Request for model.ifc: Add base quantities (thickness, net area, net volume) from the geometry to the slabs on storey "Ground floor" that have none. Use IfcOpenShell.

First a look at what the model holds.

```python
import ifcopenshell
import ifcopenshell.util.element
import ifcopenshell.util.unit

model = ifcopenshell.open("model.ifc")
print(model.schema)
for unit_type in ("LENGTHUNIT", "AREAUNIT", "VOLUMEUNIT"):
    print(unit_type, ifcopenshell.util.unit.calculate_unit_scale(model, unit_type))
storey = next(s for s in model.by_type("IfcBuildingStorey") if s.Name == "Ground floor")
slabs = [e for e in ifcopenshell.util.element.get_decomposition(storey) if e.is_a("IfcSlab")]
for e in sorted(slabs, key=lambda e: e.id()):
    print(e.id(), e.is_a(), e.Name, list(ifcopenshell.util.element.get_psets(e, qtos_only=True)), sep=" | ")
```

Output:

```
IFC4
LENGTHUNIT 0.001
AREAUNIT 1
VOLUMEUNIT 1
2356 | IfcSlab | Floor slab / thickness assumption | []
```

```python
import ifcopenshell
import ifcopenshell.api.pset
import ifcopenshell.geom
import ifcopenshell.util.element
import ifcopenshell.util.shape
import ifcopenshell.util.unit

model = ifcopenshell.open("model.ifc")
unit_scale = ifcopenshell.util.unit.calculate_unit_scale(model)
area_scale = ifcopenshell.util.unit.calculate_unit_scale(model, "AREAUNIT")
volume_scale = ifcopenshell.util.unit.calculate_unit_scale(model, "VOLUMEUNIT")
settings = ifcopenshell.geom.settings()

storey = next(s for s in model.by_type("IfcBuildingStorey") if s.Name == "Ground floor")
slabs = [e for e in ifcopenshell.util.element.get_decomposition(storey) if e.is_a("IfcSlab")]

for e in sorted(slabs, key=lambda e: e.id()):
    if ifcopenshell.util.element.get_psets(e, qtos_only=True, should_inherit=False):
        continue
    # Geometry comes back in metres, in the element's own axes.
    shape = ifcopenshell.geom.create_shape(settings, e)
    values = {
        "Width": ifcopenshell.util.shape.get_z(shape.geometry) / unit_scale,
        "NetArea": ifcopenshell.util.shape.get_footprint_area(shape.geometry) / area_scale,
        "NetVolume": ifcopenshell.util.shape.get_volume(shape.geometry) / volume_scale,
    }
    qto = ifcopenshell.api.pset.add_qto(model, product=e, name="Qto_SlabBaseQuantities")
    ifcopenshell.api.pset.edit_qto(model, qto=qto, properties=values)
    print(e.id(), {k: round(v, 3) for k, v in values.items()})

model.write("model_v2.ifc")
```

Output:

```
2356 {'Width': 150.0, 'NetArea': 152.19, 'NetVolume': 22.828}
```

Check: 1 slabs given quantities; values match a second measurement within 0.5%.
